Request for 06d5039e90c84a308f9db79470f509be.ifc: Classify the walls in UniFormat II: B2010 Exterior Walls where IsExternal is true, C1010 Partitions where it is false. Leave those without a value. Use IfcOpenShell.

First a look at what the model holds.

```python
import ifcopenshell
import ifcopenshell.util.element

model = ifcopenshell.open("06d5039e90c84a308f9db79470f509be.ifc")
print(model.schema)
print("classifications:", [c.Name for c in model.by_type("IfcClassification")])
values = [ifcopenshell.util.element.get_pset(e, "Pset_WallCommon", "IsExternal") for e in model.by_type("IfcWall")]
for value in (True, False, None):
    print("IsExternal", value, values.count(value))
```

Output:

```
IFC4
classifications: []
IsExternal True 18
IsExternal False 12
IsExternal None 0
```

```python
import ifcopenshell
import ifcopenshell.api.classification
import ifcopenshell.util.element

model = ifcopenshell.open("06d5039e90c84a308f9db79470f509be.ifc")

system = ifcopenshell.api.classification.add_classification(model, classification="UniFormat II")

walls = model.by_type("IfcWall")
external = {e: ifcopenshell.util.element.get_pset(e, "Pset_WallCommon", "IsExternal") for e in walls}
for flag, code, name in ((True, "B2010", "Exterior Walls"), (False, "C1010", "Partitions")):
    products = [e for e in walls if external[e] is flag]
    ifcopenshell.api.classification.add_reference(
        model, products=products, classification=system, identification=code, name=name
    )
    print(code, len(products))

model.write("06d5039e90c84a308f9db79470f509be-out.ifc")
```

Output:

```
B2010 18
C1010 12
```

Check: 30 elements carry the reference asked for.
